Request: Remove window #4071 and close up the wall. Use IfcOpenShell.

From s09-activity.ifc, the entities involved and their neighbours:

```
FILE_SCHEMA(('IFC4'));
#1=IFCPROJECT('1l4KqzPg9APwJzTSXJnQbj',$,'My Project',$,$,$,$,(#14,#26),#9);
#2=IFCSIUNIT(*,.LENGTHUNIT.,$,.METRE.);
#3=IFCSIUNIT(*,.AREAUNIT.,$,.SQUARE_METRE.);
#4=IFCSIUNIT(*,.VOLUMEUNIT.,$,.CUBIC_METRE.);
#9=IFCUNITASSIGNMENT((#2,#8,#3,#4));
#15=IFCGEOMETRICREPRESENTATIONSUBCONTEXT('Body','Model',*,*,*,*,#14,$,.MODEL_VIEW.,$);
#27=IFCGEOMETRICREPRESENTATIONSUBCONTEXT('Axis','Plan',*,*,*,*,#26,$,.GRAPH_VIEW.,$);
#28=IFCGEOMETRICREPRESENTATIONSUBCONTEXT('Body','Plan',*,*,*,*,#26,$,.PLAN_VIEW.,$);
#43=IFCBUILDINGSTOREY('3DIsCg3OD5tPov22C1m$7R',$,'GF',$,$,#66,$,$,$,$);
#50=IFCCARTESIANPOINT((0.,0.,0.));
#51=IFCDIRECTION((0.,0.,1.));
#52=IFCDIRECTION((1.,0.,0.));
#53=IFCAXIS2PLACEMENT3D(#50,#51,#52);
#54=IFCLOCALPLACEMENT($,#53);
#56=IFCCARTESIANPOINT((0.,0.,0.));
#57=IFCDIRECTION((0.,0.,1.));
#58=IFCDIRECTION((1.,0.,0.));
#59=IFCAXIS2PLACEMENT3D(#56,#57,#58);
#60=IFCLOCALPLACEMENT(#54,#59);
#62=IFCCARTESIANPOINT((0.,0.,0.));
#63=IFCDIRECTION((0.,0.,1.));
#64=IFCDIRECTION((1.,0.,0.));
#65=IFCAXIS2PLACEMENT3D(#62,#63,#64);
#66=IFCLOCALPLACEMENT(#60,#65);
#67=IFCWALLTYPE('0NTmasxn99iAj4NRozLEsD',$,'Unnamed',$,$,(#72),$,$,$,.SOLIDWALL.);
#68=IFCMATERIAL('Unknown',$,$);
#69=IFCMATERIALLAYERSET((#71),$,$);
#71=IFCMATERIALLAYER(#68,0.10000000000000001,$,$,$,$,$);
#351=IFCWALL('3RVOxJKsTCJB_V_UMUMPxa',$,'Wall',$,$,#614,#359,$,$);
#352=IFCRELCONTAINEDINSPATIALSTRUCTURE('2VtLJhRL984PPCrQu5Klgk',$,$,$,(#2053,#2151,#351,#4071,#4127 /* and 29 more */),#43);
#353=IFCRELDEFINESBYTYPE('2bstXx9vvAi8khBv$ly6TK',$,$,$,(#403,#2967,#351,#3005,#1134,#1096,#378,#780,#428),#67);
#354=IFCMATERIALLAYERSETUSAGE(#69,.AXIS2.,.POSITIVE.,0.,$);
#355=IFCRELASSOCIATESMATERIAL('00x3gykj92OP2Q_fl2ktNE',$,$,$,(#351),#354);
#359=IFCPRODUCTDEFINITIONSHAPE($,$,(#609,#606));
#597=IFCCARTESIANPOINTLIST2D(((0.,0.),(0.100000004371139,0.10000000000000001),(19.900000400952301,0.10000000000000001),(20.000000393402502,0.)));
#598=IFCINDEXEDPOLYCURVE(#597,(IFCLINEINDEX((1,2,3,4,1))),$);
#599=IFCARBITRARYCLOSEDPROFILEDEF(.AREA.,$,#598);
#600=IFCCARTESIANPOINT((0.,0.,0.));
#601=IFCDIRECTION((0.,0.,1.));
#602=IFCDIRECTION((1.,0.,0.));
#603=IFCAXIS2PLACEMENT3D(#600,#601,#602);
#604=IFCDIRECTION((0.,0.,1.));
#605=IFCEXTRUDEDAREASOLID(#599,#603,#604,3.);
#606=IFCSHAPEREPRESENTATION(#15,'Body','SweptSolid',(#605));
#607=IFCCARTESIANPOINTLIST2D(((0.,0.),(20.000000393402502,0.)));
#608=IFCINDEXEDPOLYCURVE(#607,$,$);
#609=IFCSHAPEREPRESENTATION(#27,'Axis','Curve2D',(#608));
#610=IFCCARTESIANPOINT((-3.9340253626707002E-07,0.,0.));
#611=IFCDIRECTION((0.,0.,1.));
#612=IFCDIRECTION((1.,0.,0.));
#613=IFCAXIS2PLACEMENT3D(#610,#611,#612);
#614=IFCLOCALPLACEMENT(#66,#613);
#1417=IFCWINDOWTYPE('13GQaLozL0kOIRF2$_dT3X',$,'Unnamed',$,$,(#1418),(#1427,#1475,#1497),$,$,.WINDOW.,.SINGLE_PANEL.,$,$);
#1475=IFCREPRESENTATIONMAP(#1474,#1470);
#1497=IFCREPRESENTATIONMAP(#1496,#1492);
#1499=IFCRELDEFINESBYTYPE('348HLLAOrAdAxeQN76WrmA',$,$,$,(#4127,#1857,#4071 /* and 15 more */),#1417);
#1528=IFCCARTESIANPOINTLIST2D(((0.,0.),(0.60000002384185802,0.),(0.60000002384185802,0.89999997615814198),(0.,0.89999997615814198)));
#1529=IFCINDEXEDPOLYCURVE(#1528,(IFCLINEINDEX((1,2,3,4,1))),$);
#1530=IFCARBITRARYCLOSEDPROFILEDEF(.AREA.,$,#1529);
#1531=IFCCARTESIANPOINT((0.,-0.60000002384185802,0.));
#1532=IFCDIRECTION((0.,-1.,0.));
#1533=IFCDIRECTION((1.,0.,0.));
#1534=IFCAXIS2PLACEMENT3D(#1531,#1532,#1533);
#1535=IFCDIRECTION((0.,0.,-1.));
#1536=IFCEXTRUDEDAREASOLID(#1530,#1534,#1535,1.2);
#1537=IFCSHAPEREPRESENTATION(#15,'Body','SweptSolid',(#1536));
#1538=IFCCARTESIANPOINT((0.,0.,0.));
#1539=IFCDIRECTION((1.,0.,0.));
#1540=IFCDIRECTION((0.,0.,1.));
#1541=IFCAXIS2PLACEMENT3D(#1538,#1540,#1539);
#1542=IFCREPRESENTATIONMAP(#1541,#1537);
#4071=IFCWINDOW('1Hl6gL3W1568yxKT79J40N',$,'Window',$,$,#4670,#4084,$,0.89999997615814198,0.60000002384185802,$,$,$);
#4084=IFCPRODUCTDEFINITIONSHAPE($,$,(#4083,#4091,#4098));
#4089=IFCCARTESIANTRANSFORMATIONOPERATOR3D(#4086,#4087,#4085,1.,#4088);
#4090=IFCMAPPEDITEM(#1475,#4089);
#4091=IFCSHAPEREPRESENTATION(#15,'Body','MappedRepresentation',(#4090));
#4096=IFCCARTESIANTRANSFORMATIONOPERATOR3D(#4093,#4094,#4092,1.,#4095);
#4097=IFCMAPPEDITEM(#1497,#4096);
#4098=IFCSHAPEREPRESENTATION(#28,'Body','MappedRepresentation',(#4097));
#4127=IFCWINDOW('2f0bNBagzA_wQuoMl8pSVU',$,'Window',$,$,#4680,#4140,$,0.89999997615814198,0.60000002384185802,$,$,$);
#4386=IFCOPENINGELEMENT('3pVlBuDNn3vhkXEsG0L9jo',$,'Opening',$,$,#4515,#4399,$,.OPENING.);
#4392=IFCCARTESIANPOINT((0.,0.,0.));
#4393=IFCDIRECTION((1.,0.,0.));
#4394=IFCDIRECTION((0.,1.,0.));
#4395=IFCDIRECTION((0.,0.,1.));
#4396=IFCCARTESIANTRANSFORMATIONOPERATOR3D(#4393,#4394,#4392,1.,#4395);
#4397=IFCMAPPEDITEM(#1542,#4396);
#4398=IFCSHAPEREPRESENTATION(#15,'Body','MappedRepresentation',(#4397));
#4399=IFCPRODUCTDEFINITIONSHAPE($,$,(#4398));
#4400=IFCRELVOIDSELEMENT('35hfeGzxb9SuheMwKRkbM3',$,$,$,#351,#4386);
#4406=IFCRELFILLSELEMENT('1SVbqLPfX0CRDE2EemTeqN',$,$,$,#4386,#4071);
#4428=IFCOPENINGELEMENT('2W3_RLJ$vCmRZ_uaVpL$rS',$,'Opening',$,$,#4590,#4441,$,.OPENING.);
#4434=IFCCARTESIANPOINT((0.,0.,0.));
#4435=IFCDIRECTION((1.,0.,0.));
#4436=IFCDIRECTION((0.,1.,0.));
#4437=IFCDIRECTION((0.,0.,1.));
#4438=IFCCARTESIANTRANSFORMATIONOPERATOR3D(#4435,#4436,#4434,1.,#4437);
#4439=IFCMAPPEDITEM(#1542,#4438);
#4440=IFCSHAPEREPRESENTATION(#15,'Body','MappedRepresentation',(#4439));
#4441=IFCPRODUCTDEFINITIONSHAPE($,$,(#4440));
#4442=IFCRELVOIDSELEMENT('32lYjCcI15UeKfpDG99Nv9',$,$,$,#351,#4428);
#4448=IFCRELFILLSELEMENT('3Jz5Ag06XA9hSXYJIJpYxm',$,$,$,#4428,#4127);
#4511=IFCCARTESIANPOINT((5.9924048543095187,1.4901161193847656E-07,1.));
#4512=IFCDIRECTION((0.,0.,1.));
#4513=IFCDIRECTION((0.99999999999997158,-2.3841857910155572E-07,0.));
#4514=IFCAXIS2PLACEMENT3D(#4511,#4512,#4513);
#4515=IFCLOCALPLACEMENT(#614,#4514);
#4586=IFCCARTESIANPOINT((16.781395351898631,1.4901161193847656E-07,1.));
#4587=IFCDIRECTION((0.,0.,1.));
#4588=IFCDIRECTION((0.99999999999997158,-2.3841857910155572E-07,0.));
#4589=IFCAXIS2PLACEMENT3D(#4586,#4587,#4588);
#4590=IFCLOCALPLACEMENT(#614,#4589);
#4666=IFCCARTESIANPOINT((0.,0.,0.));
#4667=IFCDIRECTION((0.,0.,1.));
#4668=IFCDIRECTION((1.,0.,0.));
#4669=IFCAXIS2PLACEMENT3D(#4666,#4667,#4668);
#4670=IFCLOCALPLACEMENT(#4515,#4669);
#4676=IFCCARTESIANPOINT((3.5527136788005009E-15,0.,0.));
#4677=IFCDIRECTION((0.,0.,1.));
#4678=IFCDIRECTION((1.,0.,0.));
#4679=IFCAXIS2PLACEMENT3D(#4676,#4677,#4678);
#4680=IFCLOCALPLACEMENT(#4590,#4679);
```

```python
import ifcopenshell
import ifcopenshell.api.feature
import ifcopenshell.api.root
import ifcopenshell.geom
import ifcopenshell.util.shape

model = ifcopenshell.open("s09-activity.ifc")
settings = ifcopenshell.geom.settings()


def volume(element):
    """Net volume in cubic metres, openings subtracted."""
    shape = ifcopenshell.geom.create_shape(settings, element)
    return ifcopenshell.util.shape.get_volume(shape.geometry)


window = model.by_guid("1Hl6gL3W1568yxKT79J40N")
opening = window.FillsVoids[0].RelatingOpeningElement
wall = opening.VoidsElements[0].RelatingBuildingElement
before = volume(wall)

ifcopenshell.api.root.remove_product(model, product=window)
ifcopenshell.api.feature.remove_feature(model, feature=opening)

after = volume(wall)

print(f"wall volume {before:.3f} -> {after:.3f} m3")

model.write("s09-activity-out.ifc")
```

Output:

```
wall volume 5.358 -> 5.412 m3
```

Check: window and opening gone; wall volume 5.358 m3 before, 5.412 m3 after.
